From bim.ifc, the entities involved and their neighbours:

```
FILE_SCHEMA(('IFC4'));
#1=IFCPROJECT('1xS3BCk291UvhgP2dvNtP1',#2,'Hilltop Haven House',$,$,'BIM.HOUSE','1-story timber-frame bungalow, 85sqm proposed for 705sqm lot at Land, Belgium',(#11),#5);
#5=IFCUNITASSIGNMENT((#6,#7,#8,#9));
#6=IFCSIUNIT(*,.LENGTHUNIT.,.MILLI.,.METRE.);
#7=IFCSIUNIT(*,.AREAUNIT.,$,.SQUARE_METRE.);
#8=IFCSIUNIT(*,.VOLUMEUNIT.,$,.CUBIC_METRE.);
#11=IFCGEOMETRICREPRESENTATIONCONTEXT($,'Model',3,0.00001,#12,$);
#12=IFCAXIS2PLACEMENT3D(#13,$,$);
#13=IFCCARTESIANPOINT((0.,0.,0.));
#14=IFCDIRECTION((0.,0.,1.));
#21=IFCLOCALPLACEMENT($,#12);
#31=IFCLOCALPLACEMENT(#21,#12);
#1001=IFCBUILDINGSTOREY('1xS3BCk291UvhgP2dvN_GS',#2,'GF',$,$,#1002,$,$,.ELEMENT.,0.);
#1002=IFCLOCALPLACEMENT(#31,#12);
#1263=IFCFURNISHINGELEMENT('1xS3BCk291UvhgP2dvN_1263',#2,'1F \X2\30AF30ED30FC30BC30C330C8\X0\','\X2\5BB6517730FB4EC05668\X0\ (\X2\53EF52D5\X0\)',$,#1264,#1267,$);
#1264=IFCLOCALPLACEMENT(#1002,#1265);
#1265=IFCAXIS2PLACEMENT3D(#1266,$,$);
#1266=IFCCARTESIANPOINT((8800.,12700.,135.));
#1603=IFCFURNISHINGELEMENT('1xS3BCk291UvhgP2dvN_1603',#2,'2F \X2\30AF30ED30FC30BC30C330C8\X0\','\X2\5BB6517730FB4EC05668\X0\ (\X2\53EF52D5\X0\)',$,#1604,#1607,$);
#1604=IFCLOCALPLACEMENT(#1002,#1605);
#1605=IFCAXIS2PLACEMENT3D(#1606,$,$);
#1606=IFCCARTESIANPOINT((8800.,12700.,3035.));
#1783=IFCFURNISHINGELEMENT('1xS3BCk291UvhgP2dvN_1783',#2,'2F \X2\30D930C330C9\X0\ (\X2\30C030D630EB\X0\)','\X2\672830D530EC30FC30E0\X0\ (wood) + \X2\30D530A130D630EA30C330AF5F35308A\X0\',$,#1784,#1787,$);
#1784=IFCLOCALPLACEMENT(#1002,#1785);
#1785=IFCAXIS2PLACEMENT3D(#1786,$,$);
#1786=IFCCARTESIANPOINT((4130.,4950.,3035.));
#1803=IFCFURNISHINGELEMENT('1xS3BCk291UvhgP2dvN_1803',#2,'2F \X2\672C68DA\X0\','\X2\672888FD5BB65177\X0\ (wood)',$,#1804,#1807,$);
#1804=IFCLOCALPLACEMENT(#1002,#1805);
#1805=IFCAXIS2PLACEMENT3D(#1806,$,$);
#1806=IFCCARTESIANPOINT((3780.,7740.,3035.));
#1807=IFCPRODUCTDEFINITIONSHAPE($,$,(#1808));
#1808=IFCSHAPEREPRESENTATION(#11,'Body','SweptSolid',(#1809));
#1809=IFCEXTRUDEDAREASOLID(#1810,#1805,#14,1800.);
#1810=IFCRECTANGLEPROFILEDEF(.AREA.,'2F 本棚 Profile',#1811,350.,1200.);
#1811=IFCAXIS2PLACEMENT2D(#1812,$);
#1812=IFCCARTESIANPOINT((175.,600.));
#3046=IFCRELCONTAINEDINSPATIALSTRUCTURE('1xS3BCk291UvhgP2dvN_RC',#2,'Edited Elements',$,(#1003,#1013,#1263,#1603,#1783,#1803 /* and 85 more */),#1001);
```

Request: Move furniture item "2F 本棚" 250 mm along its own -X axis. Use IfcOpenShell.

```python
import ifcopenshell
import ifcopenshell.api.geometry
import ifcopenshell.util.placement
import ifcopenshell.util.unit

model = ifcopenshell.open("bim.ifc")
unit_scale = ifcopenshell.util.unit.calculate_unit_scale(model)

item = model.by_id(1803)
matrix = ifcopenshell.util.placement.get_local_placement(item.ObjectPlacement)
matrix[:3, 3] -= matrix[:3, 0] * 0.25 / unit_scale
ifcopenshell.api.geometry.edit_object_placement(model, product=item, matrix=matrix, is_si=False)

print(ifcopenshell.util.placement.get_local_placement(item.ObjectPlacement).round(3) + 0.0)

model.write("bim_edited.ifc")
```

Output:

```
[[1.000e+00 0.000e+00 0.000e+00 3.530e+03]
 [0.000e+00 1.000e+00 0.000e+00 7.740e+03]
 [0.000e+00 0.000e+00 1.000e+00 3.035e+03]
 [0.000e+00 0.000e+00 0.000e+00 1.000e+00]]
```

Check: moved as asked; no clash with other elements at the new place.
